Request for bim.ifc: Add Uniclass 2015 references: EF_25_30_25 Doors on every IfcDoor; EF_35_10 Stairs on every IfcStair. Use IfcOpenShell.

First a look at what the model holds.

```python
import ifcopenshell

model = ifcopenshell.open("bim.ifc")
print(model.schema)
print("classifications:", [c.Name for c in model.by_type("IfcClassification")])
for ifc_class in ("IfcDoor", "IfcRoof", "IfcStair", "IfcWall", "IfcWindow"):
    print(ifc_class, len(model.by_type(ifc_class)))
```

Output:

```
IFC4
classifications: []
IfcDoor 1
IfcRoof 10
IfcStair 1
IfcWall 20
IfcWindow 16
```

```python
import ifcopenshell
import ifcopenshell.api.classification

model = ifcopenshell.open("bim.ifc")

system = ifcopenshell.api.classification.add_classification(model, classification="Uniclass 2015")

codes = {
    "IfcDoor": ("EF_25_30_25", "Doors"),
    "IfcStair": ("EF_35_10", "Stairs"),
}
for ifc_class, (code, name) in codes.items():
    products = model.by_type(ifc_class)
    ifcopenshell.api.classification.add_reference(
        model, products=products, classification=system, identification=code, name=name
    )
    print(code, len(products))

model.write("bim_rev.ifc")
```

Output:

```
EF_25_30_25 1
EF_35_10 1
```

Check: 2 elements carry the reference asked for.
